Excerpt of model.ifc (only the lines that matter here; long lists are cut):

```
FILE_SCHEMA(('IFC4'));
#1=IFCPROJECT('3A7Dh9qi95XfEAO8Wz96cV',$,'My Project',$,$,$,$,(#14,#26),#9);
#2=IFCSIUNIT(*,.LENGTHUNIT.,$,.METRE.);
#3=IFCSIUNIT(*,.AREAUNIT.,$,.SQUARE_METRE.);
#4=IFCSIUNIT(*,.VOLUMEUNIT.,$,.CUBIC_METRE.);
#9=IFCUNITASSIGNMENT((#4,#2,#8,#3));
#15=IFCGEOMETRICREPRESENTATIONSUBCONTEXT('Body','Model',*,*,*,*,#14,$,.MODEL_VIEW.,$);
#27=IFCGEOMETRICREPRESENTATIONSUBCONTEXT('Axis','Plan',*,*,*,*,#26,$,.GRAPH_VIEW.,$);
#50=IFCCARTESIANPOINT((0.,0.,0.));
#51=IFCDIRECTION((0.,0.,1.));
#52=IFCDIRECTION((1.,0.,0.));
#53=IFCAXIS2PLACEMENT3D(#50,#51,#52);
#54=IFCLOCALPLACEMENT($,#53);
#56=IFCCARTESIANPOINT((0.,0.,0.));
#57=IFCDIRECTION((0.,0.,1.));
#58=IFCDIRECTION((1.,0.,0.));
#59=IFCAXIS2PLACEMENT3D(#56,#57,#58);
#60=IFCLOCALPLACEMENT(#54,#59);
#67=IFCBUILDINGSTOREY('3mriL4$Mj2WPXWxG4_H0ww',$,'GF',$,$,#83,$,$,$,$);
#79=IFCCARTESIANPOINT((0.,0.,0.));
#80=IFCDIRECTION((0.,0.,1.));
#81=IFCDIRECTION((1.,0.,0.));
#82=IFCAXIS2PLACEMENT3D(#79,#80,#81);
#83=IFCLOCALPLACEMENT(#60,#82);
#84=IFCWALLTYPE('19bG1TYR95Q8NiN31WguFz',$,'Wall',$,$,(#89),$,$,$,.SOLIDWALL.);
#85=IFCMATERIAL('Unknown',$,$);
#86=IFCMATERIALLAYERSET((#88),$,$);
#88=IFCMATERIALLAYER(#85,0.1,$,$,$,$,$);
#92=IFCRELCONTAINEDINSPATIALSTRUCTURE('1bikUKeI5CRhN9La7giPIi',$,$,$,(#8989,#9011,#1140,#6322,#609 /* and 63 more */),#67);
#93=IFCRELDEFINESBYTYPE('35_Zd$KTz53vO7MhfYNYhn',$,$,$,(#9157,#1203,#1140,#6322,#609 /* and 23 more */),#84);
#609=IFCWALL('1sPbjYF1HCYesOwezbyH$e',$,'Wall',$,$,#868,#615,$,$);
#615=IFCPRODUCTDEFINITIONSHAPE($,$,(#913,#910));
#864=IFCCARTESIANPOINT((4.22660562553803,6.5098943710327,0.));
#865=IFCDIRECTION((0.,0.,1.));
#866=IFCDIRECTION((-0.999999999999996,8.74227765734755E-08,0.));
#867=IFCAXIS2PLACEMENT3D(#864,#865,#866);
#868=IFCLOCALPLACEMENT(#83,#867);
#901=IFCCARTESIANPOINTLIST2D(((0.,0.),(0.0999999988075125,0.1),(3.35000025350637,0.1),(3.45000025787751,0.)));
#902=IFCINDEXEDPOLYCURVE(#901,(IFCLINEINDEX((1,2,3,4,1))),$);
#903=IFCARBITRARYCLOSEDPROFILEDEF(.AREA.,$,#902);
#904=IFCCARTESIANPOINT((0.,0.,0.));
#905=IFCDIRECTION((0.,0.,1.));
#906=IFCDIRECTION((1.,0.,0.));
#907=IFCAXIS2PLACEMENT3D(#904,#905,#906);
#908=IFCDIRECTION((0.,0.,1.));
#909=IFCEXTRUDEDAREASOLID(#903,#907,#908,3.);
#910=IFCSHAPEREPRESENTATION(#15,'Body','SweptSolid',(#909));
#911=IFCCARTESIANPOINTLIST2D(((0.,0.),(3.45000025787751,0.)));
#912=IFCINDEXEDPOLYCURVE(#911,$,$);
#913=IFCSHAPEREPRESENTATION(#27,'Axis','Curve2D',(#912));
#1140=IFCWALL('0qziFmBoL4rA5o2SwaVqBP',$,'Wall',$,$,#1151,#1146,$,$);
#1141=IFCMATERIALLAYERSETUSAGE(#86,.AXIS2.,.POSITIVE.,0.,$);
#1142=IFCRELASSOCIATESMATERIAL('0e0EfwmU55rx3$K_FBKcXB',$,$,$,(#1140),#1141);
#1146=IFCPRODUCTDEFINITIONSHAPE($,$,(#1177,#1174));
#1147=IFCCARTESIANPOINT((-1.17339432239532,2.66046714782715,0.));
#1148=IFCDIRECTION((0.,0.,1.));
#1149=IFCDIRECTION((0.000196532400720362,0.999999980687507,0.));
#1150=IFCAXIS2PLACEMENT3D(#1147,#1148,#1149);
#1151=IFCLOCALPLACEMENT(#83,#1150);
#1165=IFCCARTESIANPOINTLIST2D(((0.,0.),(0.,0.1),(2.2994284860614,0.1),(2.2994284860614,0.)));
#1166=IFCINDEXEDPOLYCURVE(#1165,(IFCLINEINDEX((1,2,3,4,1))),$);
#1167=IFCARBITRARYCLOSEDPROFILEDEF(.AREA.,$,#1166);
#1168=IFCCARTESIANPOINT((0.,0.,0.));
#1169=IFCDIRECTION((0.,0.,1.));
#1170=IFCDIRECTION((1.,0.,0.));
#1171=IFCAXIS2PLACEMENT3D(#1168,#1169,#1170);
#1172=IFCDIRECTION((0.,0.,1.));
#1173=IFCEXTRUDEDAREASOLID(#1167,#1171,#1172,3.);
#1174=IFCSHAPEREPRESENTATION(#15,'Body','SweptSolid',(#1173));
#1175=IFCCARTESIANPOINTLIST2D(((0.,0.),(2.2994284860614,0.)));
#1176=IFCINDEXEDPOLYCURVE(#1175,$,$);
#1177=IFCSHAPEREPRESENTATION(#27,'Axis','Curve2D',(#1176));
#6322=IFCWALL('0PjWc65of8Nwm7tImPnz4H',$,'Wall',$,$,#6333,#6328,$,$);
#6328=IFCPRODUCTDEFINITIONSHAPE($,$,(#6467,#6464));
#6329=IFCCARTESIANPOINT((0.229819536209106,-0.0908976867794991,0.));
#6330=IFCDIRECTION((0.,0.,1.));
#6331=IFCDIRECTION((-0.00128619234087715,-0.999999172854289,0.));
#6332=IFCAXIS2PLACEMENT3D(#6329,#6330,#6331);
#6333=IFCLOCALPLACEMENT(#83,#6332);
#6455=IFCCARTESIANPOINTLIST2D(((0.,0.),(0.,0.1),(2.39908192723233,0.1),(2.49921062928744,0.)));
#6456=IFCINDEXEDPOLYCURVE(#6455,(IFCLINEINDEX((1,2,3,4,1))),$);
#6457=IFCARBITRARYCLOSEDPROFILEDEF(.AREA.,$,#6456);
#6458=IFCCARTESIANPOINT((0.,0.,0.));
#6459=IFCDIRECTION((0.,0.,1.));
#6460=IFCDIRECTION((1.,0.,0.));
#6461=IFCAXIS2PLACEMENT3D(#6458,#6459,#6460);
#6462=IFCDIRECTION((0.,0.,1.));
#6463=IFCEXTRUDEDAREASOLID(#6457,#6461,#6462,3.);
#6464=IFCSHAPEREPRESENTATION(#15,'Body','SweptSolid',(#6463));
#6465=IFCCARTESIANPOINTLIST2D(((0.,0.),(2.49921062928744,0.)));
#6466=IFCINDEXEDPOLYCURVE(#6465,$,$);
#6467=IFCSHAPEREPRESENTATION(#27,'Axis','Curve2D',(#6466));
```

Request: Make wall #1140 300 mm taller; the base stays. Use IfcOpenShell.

```python
import ifcopenshell
import ifcopenshell.geom
import ifcopenshell.util.representation
import ifcopenshell.util.shape
import ifcopenshell.util.unit

model = ifcopenshell.open("model.ifc")
unit_scale = ifcopenshell.util.unit.calculate_unit_scale(model)
settings = ifcopenshell.geom.settings()


def volume(element):
    """Net volume in cubic metres, openings subtracted."""
    shape = ifcopenshell.geom.create_shape(settings, element)
    return ifcopenshell.util.shape.get_volume(shape.geometry)


wall = model.by_id(1140)
before = volume(wall)

body = ifcopenshell.util.representation.get_representation(wall, "Model", "Body")
solid = body.Items[0]
old_height = solid.Depth
solid.Depth += 0.3 / unit_scale
after = volume(wall)

print(f"height {old_height:g} -> {solid.Depth:g}, volume {before:.3f} -> {after:.3f} m3")

model.write("model_edited.ifc")
```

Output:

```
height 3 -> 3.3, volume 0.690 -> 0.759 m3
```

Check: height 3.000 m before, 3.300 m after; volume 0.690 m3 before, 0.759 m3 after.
